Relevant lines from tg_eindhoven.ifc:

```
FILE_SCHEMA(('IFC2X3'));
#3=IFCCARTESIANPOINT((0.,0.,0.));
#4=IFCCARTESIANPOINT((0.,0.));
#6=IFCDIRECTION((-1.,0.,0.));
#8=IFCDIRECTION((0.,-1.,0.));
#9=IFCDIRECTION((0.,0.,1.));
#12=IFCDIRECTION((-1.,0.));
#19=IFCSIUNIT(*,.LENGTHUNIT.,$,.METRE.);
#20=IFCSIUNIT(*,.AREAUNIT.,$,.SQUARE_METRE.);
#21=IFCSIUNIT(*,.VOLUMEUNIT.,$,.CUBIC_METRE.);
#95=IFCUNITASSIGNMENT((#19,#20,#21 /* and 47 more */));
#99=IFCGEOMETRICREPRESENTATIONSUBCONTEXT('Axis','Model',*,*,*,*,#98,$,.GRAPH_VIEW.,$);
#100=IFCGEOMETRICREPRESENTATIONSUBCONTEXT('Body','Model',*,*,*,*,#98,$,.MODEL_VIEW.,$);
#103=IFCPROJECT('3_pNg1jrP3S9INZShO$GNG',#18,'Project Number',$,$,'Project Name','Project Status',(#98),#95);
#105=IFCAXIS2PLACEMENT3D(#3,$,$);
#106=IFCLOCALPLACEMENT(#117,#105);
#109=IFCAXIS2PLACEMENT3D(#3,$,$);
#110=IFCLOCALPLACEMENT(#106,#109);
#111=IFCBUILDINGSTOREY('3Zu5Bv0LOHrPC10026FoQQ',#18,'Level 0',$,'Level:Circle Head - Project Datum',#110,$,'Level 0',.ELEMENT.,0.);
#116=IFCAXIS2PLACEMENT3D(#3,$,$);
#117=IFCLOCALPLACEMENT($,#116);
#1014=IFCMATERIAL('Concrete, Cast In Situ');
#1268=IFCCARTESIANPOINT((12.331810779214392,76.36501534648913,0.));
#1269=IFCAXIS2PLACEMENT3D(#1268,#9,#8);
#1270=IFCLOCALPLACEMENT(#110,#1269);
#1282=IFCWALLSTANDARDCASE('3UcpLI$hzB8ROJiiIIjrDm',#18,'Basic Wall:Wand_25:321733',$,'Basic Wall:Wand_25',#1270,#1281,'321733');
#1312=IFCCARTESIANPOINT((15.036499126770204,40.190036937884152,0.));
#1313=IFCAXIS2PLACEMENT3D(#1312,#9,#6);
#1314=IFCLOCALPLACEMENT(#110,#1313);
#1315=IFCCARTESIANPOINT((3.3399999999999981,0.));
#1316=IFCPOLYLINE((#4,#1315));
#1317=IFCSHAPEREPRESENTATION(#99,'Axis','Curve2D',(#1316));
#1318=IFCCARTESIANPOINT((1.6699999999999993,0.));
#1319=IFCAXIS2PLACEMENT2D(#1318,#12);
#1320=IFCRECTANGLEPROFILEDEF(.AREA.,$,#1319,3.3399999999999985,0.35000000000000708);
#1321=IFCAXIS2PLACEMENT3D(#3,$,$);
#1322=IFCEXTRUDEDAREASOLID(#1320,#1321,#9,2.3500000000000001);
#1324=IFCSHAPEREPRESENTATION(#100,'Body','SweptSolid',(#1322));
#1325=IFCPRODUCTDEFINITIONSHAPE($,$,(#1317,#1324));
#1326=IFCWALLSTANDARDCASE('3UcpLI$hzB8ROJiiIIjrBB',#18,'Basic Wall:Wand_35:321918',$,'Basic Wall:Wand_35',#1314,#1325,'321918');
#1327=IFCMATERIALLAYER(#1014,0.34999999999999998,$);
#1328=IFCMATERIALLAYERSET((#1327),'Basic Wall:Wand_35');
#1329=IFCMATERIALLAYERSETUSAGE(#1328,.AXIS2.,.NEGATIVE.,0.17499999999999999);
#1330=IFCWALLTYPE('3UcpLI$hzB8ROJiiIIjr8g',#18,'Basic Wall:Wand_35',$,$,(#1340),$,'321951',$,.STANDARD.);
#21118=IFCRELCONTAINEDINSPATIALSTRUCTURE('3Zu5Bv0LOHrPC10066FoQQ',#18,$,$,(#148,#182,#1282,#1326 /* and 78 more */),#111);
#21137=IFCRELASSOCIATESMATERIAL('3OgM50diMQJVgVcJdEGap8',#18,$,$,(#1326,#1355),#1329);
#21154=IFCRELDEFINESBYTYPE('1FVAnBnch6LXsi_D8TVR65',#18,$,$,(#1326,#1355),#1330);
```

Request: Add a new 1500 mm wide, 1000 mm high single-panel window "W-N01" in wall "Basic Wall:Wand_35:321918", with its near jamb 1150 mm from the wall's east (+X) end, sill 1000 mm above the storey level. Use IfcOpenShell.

```python
import numpy as np
import ifcopenshell
import ifcopenshell.api.feature
import ifcopenshell.api.geometry
import ifcopenshell.api.root
import ifcopenshell.api.spatial
import ifcopenshell.api.type
import ifcopenshell.geom
import ifcopenshell.util.element
import ifcopenshell.util.placement
import ifcopenshell.util.representation
import ifcopenshell.util.shape
import ifcopenshell.util.unit

model = ifcopenshell.open("tg_eindhoven.ifc")
unit_scale = ifcopenshell.util.unit.calculate_unit_scale(model)
settings = ifcopenshell.geom.settings()


def volume(element):
    """Net volume in cubic metres, openings subtracted."""
    shape = ifcopenshell.geom.create_shape(settings, element)
    return ifcopenshell.util.shape.get_volume(shape.geometry)


wall = model.by_id(1326)
storey = ifcopenshell.util.element.get_container(wall, ifc_class="IfcBuildingStorey")
context = ifcopenshell.util.representation.get_context(model, "Model", "Body", "MODEL_VIEW")
before = volume(wall)

width, height, from_end, sill = 1.5, 1, 1.15, 1  # metres

# The wall runs along its own X axis, and the end named is its -X end.
wall_shape = ifcopenshell.geom.create_shape(settings, wall)
x, y, z = ifcopenshell.util.shape.get_vertices(wall_shape.geometry).T
start = x.min() + from_end
face, thickness = float(y.min()), float(y.max() - y.min())
wall_matrix = ifcopenshell.util.placement.get_local_placement(wall.ObjectPlacement)
level = ifcopenshell.util.placement.get_local_placement(storey.ObjectPlacement)[2, 3]


def in_wall(x, y):
    """Placement at x, y metres in the wall's axes, at sill height."""
    matrix = wall_matrix.copy()
    matrix[:, 3] = wall_matrix @ np.array([x / unit_scale, y / unit_scale, 0.0, 1.0])
    matrix[2, 3] = level + sill / unit_scale
    return matrix


# Opening: a box that overshoots both wall faces by 50 mm.
opening = ifcopenshell.api.root.create_entity(model, ifc_class="IfcOpeningElement")
box = ifcopenshell.api.geometry.add_wall_representation(
    model, context=context, length=width, height=height, thickness=thickness + 0.1
)
ifcopenshell.api.geometry.assign_representation(model, product=opening, representation=box)
ifcopenshell.api.geometry.edit_object_placement(model, product=opening, matrix=in_wall(start, face - 0.05), is_si=False)
ifcopenshell.api.feature.add_feature(model, feature=opening, element=wall)

window = ifcopenshell.api.root.create_entity(model, ifc_class="IfcWindow", name="W-N01")
window.OverallWidth, window.OverallHeight = width / unit_scale, height / unit_scale
body = ifcopenshell.api.geometry.add_window_representation(
    model,
    context=context,
    overall_width=window.OverallWidth,
    overall_height=window.OverallHeight,
    partition_type="SINGLE_PANEL",
)
ifcopenshell.api.geometry.assign_representation(model, product=window, representation=body)
ifcopenshell.api.spatial.assign_container(model, products=[window], relating_structure=storey)
fills = ifcopenshell.api.feature.add_filling(model, opening=opening, element=window)
fills.OwnerHistory = window.OwnerHistory  # required in IFC2X3

# IFC2X3 keeps the operation on the window style.
style = ifcopenshell.api.root.create_entity(model, ifc_class="IfcWindowStyle", name="W-N01")
style.OperationType, style.ConstructionType = "SINGLE_PANEL", "NOTDEFINED"
style.ParameterTakesPrecedence = style.Sizeable = False
ifcopenshell.api.type.assign_type(model, related_objects=[window], relating_type=style)

# Centre the window in the wall's thickness.
ifcopenshell.api.geometry.edit_object_placement(model, product=window, matrix=in_wall(start, face), is_si=False)
window_shape = ifcopenshell.geom.create_shape(settings, window)
depth = ifcopenshell.util.shape.get_vertices(window_shape.geometry)[:, 1]
offset = face + thickness / 2 - (depth.min() + depth.max()) / 2
ifcopenshell.api.geometry.edit_object_placement(model, product=window, matrix=in_wall(start, offset), is_si=False)

after = volume(wall)

print(f"wall volume {before:.3f} -> {after:.3f} m3")

model.write("tg_eindhoven-out.ifc")
```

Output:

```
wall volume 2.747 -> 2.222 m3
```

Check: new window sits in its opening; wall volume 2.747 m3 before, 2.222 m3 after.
